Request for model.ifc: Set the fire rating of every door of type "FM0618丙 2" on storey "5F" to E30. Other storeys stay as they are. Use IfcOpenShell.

First a look at what the model holds.

```python
import ifcopenshell
import ifcopenshell.util.element

model = ifcopenshell.open("model.ifc")
print(model.schema)
storey = next(s for s in model.by_type("IfcBuildingStorey") if s.Name == "5F")
doors = [e for e in ifcopenshell.util.element.get_decomposition(storey) if e.is_a("IfcDoor")]
seen = {}
for e in doors:
    element_type = ifcopenshell.util.element.get_type(e)
    key = (element_type.Name if element_type != e and element_type else None, ifcopenshell.util.element.get_pset(e, "Pset_DoorCommon", "FireRating"))
    seen[key] = seen.get(key, 0) + 1
for (name, value), count in sorted(seen.items(), key=str):
    print(count, "x", name, "|", value)
```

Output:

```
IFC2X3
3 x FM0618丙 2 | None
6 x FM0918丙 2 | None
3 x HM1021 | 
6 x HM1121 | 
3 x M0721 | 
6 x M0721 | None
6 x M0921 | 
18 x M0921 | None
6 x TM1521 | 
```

```python
import ifcopenshell
import ifcopenshell.api.pset
import ifcopenshell.util.element

model = ifcopenshell.open("model.ifc")

storey = next(s for s in model.by_type("IfcBuildingStorey") if s.Name == "5F")
doors = [e for e in ifcopenshell.util.element.get_decomposition(storey) if e.is_a("IfcDoor")]

count = 0
for e in doors:
    element_type = ifcopenshell.util.element.get_type(e)
    if element_type in (None, e) or element_type.Name != "FM0618丙 2":
        continue
    # add_pset returns the element's existing set when there is one.
    pset = ifcopenshell.api.pset.add_pset(model, product=e, name="Pset_DoorCommon")
    ifcopenshell.api.pset.edit_pset(model, pset=pset, properties={"FireRating": "E30"})
    count += 1

print(count, "doors updated")

model.write("model-out.ifc")
```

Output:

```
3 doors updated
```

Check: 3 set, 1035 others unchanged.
